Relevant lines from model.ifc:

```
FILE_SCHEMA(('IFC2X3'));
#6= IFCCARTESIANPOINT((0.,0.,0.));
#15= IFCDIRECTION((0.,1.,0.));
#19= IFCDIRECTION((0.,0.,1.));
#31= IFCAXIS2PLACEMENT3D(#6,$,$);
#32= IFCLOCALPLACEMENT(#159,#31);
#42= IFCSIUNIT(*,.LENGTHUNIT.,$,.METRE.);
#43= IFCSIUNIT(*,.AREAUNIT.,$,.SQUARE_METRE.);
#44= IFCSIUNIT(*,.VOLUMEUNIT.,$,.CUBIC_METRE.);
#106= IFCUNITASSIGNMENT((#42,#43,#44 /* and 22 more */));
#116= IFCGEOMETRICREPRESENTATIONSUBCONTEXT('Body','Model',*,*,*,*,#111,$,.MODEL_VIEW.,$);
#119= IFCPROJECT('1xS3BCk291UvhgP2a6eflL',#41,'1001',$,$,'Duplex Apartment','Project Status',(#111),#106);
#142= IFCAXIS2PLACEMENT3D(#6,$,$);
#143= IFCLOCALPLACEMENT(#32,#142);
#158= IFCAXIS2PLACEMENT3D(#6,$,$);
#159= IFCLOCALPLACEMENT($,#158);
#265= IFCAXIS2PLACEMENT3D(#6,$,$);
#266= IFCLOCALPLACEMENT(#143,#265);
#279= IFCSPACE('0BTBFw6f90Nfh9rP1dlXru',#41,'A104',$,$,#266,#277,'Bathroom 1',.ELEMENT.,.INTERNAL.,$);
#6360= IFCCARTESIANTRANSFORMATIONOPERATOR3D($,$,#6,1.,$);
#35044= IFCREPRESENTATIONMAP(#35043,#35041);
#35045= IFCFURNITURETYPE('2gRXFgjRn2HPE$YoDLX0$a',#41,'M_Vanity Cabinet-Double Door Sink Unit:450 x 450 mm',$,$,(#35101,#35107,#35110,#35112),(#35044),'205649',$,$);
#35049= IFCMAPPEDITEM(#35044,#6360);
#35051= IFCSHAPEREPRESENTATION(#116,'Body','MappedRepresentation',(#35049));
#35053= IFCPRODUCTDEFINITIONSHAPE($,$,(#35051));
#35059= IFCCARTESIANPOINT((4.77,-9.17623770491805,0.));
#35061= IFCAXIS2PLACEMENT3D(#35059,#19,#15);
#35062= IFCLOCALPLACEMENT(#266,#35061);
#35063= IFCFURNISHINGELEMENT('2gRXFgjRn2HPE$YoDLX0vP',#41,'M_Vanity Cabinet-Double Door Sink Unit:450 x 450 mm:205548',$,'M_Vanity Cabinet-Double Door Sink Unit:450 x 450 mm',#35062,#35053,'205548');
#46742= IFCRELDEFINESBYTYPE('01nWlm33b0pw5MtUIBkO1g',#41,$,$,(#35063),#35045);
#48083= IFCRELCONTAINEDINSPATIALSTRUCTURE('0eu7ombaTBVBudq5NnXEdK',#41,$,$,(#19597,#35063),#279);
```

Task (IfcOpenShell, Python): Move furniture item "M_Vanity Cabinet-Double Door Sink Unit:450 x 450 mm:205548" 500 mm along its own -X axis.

```python
import ifcopenshell
import ifcopenshell.api.geometry
import ifcopenshell.util.placement
import ifcopenshell.util.unit

model = ifcopenshell.open("model.ifc")
unit_scale = ifcopenshell.util.unit.calculate_unit_scale(model)

item = model.by_guid("2gRXFgjRn2HPE$YoDLX0vP")
matrix = ifcopenshell.util.placement.get_local_placement(item.ObjectPlacement)
matrix[:3, 3] -= matrix[:3, 0] * 0.5 / unit_scale
ifcopenshell.api.geometry.edit_object_placement(model, product=item, matrix=matrix, is_si=False)

print(ifcopenshell.util.placement.get_local_placement(item.ObjectPlacement).round(3) + 0.0)

model.write("model_edited.ifc")
```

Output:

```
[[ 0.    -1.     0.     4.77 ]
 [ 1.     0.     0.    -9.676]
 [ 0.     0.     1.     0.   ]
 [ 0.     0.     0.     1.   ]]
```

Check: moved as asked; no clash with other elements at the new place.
